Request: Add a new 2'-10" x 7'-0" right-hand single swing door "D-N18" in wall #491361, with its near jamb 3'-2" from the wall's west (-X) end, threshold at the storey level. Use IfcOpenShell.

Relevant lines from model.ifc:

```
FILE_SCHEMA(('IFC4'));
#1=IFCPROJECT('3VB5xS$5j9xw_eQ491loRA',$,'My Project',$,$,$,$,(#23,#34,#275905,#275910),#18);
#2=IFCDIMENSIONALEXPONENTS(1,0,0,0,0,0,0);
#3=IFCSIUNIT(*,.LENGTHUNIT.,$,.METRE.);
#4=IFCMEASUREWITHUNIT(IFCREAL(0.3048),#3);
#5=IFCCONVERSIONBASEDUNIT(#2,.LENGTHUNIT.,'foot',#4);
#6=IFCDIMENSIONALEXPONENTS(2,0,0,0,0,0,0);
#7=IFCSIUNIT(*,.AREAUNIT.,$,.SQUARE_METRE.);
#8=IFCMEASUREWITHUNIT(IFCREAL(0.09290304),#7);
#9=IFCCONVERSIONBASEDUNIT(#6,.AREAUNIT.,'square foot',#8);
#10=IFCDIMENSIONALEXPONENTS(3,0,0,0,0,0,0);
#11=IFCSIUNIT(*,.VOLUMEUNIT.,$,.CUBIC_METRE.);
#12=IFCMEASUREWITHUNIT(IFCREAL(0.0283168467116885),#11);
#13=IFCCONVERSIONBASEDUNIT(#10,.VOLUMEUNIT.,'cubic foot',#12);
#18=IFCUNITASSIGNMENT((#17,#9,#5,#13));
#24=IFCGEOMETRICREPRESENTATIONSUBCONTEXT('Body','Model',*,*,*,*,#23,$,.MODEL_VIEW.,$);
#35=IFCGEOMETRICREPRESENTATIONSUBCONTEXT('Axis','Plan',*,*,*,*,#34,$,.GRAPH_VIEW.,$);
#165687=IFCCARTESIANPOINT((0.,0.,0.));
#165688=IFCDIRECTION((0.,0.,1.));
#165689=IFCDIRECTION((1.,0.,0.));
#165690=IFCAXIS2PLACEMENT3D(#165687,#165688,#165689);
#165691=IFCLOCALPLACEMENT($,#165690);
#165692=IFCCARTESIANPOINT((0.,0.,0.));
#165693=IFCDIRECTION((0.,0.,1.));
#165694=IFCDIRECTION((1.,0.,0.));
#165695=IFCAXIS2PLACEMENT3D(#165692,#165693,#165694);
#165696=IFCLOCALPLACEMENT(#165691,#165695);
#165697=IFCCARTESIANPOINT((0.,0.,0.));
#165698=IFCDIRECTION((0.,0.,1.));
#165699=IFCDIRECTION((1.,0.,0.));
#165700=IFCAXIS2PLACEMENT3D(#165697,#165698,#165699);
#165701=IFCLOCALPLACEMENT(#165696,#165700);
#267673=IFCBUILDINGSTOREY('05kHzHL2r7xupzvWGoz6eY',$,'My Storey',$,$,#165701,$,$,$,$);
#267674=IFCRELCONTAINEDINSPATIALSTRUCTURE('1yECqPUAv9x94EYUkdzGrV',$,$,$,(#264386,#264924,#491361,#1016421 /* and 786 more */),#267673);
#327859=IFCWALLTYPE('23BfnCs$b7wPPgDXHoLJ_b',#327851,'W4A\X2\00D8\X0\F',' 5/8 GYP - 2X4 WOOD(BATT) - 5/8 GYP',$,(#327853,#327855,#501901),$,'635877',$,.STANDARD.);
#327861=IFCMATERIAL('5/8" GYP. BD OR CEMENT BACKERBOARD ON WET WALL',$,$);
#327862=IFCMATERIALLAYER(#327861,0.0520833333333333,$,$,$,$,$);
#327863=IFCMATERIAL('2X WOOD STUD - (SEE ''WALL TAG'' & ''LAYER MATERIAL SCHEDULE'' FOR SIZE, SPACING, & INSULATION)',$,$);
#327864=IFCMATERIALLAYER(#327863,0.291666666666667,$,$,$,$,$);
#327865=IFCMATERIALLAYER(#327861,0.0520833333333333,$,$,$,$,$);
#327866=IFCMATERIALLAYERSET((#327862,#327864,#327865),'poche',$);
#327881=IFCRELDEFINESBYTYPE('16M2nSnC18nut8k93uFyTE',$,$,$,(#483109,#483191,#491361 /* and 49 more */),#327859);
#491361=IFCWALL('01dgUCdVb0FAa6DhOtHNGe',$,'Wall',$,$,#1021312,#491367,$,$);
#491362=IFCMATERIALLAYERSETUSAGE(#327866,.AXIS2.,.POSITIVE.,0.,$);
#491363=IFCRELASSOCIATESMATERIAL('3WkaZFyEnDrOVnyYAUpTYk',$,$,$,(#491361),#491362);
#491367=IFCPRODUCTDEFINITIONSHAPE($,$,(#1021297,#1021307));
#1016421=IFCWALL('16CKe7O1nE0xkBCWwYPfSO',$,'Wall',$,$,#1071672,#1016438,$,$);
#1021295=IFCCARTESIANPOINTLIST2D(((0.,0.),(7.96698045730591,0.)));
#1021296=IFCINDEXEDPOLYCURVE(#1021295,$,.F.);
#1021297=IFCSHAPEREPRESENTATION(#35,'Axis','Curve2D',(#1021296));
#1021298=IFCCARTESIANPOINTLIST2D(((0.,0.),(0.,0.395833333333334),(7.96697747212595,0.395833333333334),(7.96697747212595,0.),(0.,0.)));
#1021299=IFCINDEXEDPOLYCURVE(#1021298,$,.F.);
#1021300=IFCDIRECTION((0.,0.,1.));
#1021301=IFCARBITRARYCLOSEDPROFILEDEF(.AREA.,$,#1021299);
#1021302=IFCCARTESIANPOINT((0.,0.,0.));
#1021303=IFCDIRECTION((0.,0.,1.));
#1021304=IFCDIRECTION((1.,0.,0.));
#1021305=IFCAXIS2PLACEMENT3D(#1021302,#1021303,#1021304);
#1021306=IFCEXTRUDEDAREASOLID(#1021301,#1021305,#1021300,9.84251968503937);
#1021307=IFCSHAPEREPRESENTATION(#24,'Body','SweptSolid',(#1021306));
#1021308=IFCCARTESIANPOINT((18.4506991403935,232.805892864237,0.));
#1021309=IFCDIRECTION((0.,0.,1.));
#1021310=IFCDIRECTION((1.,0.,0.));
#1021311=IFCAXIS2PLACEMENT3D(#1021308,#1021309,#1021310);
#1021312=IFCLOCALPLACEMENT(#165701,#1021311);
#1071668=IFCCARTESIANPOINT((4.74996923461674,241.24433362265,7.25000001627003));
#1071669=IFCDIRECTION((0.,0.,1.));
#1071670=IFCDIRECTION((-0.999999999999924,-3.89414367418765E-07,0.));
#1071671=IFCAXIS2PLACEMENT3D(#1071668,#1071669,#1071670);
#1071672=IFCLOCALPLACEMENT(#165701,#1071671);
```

```python
import numpy as np
import ifcopenshell
import ifcopenshell.api.feature
import ifcopenshell.api.geometry
import ifcopenshell.api.root
import ifcopenshell.api.spatial
import ifcopenshell.geom
import ifcopenshell.util.element
import ifcopenshell.util.placement
import ifcopenshell.util.representation
import ifcopenshell.util.shape
import ifcopenshell.util.unit

model = ifcopenshell.open("model.ifc")
unit_scale = ifcopenshell.util.unit.calculate_unit_scale(model)
settings = ifcopenshell.geom.settings()


def volume(element):
    """Net volume in cubic metres, openings subtracted."""
    shape = ifcopenshell.geom.create_shape(settings, element)
    return ifcopenshell.util.shape.get_volume(shape.geometry)


wall = model.by_guid("01dgUCdVb0FAa6DhOtHNGe")
storey = ifcopenshell.util.element.get_container(wall, ifc_class="IfcBuildingStorey")
context = ifcopenshell.util.representation.get_context(model, "Model", "Body", "MODEL_VIEW")
before = volume(wall)

width, height, from_end, sill = 0.8636, 2.1336, 0.9652, 0.0  # metres

# The wall runs along its own X axis, and the end named is its -X end.
wall_shape = ifcopenshell.geom.create_shape(settings, wall)
x, y, z = ifcopenshell.util.shape.get_vertices(wall_shape.geometry).T
start = x.min() + from_end
face, thickness = float(y.min()), float(y.max() - y.min())
wall_matrix = ifcopenshell.util.placement.get_local_placement(wall.ObjectPlacement)
level = ifcopenshell.util.placement.get_local_placement(storey.ObjectPlacement)[2, 3]


def in_wall(x, y):
    """Placement at x, y metres in the wall's axes, at sill height."""
    matrix = wall_matrix.copy()
    matrix[:, 3] = wall_matrix @ np.array([x / unit_scale, y / unit_scale, 0.0, 1.0])
    matrix[2, 3] = level + sill / unit_scale
    return matrix


# Opening: a box that overshoots both wall faces by 50 mm.
opening = ifcopenshell.api.root.create_entity(model, ifc_class="IfcOpeningElement", predefined_type="OPENING")
box = ifcopenshell.api.geometry.add_wall_representation(
    model, context=context, length=width, height=height, thickness=thickness + 0.1
)
ifcopenshell.api.geometry.assign_representation(model, product=opening, representation=box)
ifcopenshell.api.geometry.edit_object_placement(model, product=opening, matrix=in_wall(start, face - 0.05), is_si=False)
ifcopenshell.api.feature.add_feature(model, feature=opening, element=wall)

door = ifcopenshell.api.root.create_entity(model, ifc_class="IfcDoor", name="D-N18", predefined_type="DOOR")
door.OverallWidth, door.OverallHeight = width / unit_scale, height / unit_scale
door.OperationType = "SINGLE_SWING_RIGHT"
body = ifcopenshell.api.geometry.add_door_representation(
    model,
    context=context,
    overall_width=door.OverallWidth,
    overall_height=door.OverallHeight,
    operation_type="SINGLE_SWING_RIGHT",
    lining_properties={"LiningDepth": thickness / unit_scale, "ThresholdDepth": thickness / unit_scale},
)
ifcopenshell.api.geometry.assign_representation(model, product=door, representation=body)
ifcopenshell.api.spatial.assign_container(model, products=[door], relating_structure=storey)
ifcopenshell.api.feature.add_filling(model, opening=opening, element=door)

# The lining spans the wall, so the door starts at the wall face.
ifcopenshell.api.geometry.edit_object_placement(model, product=door, matrix=in_wall(start, face), is_si=False)

after = volume(wall)

print(f"wall volume {before:.3f} -> {after:.3f} m3")

model.write("model_edited.ifc")
```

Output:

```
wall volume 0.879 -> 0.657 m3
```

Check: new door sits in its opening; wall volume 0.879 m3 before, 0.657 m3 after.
